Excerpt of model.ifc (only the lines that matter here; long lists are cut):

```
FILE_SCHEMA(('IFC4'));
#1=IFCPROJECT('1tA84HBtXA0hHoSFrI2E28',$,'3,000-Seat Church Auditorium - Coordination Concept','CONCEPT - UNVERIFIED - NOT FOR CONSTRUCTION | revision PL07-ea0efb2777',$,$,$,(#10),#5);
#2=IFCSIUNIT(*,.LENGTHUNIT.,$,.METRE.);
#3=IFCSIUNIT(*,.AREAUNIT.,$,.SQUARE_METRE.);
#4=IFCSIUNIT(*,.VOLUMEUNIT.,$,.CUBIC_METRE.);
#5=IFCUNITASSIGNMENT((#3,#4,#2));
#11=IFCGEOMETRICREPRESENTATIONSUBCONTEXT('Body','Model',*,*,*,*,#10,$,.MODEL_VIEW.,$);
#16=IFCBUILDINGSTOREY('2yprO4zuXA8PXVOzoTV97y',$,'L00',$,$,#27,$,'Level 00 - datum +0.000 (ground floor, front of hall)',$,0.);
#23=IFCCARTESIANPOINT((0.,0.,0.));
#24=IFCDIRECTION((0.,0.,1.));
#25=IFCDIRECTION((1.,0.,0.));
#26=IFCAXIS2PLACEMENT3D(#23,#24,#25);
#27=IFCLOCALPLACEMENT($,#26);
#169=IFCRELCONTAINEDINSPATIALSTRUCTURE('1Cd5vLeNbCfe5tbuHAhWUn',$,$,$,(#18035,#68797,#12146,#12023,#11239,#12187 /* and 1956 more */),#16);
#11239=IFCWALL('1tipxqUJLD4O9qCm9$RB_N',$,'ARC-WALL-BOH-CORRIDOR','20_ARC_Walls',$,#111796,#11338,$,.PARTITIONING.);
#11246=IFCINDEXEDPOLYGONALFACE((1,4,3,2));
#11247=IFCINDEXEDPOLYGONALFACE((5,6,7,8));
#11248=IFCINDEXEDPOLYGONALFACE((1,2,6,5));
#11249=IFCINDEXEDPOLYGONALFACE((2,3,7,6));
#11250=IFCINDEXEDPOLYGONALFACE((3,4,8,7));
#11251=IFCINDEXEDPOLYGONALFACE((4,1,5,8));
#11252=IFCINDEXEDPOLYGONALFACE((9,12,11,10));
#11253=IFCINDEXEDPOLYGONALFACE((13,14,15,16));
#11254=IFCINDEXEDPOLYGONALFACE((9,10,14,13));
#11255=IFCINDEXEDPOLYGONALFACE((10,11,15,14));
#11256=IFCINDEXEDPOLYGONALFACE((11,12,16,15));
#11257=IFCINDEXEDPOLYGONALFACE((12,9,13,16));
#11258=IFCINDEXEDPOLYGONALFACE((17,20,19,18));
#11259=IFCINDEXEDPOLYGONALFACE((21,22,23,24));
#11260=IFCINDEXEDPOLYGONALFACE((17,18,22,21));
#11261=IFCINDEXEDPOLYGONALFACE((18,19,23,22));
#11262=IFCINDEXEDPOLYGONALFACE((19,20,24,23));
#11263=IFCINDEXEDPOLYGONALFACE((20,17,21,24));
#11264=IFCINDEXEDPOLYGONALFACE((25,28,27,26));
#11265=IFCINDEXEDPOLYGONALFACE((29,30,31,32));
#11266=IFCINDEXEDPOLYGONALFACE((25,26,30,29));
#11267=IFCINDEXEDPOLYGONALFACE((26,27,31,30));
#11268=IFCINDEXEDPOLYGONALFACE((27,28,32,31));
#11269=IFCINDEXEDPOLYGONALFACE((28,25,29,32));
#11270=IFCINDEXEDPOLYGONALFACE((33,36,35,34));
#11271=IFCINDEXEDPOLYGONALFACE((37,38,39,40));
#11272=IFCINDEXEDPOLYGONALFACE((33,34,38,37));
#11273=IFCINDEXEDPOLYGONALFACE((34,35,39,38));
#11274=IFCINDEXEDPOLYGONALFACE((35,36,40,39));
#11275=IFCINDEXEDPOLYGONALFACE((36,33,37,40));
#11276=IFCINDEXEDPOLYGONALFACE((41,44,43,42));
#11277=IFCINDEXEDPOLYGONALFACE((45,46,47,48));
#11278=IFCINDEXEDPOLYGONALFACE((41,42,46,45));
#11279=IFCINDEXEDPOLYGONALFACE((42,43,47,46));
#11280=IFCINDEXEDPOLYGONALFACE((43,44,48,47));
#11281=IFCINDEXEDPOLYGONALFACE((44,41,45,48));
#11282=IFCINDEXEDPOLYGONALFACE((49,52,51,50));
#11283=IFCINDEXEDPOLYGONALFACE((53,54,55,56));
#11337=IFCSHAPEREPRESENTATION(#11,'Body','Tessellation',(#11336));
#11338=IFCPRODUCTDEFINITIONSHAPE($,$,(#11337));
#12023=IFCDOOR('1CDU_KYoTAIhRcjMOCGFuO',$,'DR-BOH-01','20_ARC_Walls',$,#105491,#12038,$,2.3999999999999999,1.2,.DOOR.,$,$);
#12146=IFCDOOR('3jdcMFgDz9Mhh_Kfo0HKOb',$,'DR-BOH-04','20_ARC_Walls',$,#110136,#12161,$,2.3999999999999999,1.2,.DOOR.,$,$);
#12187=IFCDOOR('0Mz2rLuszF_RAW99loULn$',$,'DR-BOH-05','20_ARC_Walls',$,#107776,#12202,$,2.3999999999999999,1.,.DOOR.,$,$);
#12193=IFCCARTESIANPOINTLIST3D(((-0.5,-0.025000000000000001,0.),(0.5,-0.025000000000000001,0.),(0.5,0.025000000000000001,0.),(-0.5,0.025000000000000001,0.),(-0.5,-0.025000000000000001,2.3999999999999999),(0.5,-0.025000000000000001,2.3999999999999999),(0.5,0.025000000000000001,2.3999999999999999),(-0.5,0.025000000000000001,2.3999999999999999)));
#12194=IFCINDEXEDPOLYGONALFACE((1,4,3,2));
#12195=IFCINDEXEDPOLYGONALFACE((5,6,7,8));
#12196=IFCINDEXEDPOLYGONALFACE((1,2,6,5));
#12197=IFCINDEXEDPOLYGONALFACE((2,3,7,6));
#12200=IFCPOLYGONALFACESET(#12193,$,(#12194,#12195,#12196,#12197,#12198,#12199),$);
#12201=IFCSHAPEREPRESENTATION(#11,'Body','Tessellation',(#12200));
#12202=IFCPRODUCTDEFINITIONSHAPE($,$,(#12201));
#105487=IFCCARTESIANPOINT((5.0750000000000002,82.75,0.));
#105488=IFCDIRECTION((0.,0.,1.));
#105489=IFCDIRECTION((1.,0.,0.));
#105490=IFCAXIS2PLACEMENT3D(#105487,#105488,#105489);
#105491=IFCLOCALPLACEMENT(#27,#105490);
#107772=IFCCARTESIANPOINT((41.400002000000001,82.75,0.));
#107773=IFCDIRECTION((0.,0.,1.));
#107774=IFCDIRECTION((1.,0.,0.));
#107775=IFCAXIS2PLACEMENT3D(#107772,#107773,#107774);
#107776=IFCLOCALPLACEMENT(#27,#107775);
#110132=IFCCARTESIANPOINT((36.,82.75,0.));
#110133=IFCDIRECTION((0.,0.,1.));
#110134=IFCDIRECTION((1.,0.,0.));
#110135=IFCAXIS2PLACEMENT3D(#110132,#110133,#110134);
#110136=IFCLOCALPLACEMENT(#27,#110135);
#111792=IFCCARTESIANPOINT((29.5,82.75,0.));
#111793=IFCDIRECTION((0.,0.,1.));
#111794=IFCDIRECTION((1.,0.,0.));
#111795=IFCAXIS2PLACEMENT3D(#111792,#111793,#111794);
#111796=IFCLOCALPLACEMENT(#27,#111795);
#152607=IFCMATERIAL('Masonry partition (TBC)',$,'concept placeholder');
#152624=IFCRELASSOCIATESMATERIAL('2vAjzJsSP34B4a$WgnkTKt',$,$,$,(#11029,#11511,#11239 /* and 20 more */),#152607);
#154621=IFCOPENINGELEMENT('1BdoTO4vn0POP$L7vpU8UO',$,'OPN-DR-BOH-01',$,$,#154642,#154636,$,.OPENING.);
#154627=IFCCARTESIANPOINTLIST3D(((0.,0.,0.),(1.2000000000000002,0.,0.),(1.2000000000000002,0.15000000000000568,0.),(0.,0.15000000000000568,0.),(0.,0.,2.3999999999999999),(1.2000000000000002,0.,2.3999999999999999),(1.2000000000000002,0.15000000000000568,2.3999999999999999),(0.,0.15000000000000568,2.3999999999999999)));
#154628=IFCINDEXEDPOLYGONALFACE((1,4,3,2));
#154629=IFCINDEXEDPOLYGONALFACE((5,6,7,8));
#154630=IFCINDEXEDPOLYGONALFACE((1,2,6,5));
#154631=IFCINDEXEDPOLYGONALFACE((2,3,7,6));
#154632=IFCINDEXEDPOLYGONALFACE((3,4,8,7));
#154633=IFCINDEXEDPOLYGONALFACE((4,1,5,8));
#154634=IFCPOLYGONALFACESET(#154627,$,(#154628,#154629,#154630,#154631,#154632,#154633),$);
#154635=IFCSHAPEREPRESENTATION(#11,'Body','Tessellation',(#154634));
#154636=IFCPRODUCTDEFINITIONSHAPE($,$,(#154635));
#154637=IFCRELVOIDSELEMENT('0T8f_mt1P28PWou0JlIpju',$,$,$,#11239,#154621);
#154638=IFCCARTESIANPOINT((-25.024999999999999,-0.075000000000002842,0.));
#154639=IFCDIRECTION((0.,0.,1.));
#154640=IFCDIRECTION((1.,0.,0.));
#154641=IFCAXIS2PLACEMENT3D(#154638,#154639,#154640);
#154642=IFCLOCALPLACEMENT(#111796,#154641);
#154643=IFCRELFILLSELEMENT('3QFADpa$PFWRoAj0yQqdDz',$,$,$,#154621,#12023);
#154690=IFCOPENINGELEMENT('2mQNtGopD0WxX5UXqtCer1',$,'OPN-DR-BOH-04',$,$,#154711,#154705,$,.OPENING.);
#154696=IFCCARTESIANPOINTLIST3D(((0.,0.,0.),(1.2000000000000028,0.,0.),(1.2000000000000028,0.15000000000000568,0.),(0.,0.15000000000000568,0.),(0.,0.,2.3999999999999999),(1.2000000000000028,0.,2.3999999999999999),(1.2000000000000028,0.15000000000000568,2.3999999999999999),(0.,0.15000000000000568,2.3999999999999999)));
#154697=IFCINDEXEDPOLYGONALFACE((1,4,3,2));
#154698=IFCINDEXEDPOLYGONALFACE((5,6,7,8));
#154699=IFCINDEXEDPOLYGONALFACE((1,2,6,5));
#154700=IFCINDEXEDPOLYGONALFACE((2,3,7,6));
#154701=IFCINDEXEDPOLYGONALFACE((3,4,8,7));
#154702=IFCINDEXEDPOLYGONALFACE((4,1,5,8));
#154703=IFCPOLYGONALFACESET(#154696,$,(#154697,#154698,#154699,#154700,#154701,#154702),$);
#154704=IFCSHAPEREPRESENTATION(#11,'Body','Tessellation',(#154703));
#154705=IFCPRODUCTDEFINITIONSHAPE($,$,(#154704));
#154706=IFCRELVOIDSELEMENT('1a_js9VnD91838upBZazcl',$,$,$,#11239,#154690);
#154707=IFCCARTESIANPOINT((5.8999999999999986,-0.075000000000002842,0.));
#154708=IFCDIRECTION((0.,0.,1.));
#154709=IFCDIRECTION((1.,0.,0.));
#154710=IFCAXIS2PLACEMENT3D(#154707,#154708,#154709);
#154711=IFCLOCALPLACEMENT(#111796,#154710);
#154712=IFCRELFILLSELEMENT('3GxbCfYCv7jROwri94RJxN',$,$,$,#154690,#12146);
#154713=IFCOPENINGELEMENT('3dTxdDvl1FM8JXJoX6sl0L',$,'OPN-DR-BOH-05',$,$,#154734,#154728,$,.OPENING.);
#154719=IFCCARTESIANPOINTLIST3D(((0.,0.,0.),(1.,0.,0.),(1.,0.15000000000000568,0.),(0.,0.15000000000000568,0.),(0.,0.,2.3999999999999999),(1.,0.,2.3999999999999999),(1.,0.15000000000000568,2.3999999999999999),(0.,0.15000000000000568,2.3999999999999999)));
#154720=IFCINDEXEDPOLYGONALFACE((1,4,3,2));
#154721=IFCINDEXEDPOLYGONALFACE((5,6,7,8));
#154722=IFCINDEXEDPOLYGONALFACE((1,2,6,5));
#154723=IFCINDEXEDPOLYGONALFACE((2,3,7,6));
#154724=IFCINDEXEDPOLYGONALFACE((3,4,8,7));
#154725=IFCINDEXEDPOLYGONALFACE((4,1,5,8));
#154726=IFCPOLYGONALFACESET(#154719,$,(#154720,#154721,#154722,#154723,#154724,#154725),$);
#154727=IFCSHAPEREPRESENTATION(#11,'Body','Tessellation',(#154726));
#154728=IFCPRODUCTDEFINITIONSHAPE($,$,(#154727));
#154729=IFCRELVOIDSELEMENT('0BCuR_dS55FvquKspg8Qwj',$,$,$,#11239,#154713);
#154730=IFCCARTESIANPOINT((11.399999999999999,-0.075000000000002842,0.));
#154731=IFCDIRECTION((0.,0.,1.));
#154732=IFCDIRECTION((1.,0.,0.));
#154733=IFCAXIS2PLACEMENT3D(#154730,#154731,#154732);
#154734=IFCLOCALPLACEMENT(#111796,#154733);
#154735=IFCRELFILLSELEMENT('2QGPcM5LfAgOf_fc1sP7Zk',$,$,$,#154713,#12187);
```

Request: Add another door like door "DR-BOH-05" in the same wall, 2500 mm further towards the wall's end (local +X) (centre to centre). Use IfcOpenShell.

```python
import ifcopenshell
import ifcopenshell.api.feature
import ifcopenshell.api.geometry
import ifcopenshell.api.root
import ifcopenshell.geom
import ifcopenshell.util.element
import ifcopenshell.util.placement
import ifcopenshell.util.shape

model = ifcopenshell.open("model.ifc")
settings = ifcopenshell.geom.settings()


def volume(element):
    """Net volume in cubic metres, openings subtracted."""
    shape = ifcopenshell.geom.create_shape(settings, element)
    return ifcopenshell.util.shape.get_volume(shape.geometry)


door = model.by_guid("0Mz2rLuszF_RAW99loULn$")
opening = door.FillsVoids[0].RelatingOpeningElement
wall = opening.VoidsElements[0].RelatingBuildingElement
before = volume(wall)
shift = ifcopenshell.util.placement.get_local_placement(wall.ObjectPlacement)[:3, 0] * 2.5

# copy_class copies the void relationship, type, container and properties, but no geometry.
new_opening = ifcopenshell.api.root.copy_class(model, product=opening)
new_opening.Representation = ifcopenshell.util.element.copy_deep(
    model, opening.Representation, exclude=["IfcGeometricRepresentationContext", "IfcRepresentationMap"]
)
new_door = ifcopenshell.api.root.copy_class(model, product=door)
new_door.Representation = ifcopenshell.util.element.copy_deep(
    model, door.Representation, exclude=["IfcGeometricRepresentationContext", "IfcRepresentationMap"]
)
ifcopenshell.api.feature.add_filling(model, opening=new_opening, element=new_door)

for old, new in ((opening, new_opening), (door, new_door)):
    matrix = ifcopenshell.util.placement.get_local_placement(old.ObjectPlacement)
    matrix[:3, 3] += shift
    ifcopenshell.api.geometry.edit_object_placement(model, product=new, matrix=matrix, is_si=False)

after = volume(wall)

print(f"wall volume {before:.3f} -> {after:.3f} m3")

model.write("model_edited.ifc")
```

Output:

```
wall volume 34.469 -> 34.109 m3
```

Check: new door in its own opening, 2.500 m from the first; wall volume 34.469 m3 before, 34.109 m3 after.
